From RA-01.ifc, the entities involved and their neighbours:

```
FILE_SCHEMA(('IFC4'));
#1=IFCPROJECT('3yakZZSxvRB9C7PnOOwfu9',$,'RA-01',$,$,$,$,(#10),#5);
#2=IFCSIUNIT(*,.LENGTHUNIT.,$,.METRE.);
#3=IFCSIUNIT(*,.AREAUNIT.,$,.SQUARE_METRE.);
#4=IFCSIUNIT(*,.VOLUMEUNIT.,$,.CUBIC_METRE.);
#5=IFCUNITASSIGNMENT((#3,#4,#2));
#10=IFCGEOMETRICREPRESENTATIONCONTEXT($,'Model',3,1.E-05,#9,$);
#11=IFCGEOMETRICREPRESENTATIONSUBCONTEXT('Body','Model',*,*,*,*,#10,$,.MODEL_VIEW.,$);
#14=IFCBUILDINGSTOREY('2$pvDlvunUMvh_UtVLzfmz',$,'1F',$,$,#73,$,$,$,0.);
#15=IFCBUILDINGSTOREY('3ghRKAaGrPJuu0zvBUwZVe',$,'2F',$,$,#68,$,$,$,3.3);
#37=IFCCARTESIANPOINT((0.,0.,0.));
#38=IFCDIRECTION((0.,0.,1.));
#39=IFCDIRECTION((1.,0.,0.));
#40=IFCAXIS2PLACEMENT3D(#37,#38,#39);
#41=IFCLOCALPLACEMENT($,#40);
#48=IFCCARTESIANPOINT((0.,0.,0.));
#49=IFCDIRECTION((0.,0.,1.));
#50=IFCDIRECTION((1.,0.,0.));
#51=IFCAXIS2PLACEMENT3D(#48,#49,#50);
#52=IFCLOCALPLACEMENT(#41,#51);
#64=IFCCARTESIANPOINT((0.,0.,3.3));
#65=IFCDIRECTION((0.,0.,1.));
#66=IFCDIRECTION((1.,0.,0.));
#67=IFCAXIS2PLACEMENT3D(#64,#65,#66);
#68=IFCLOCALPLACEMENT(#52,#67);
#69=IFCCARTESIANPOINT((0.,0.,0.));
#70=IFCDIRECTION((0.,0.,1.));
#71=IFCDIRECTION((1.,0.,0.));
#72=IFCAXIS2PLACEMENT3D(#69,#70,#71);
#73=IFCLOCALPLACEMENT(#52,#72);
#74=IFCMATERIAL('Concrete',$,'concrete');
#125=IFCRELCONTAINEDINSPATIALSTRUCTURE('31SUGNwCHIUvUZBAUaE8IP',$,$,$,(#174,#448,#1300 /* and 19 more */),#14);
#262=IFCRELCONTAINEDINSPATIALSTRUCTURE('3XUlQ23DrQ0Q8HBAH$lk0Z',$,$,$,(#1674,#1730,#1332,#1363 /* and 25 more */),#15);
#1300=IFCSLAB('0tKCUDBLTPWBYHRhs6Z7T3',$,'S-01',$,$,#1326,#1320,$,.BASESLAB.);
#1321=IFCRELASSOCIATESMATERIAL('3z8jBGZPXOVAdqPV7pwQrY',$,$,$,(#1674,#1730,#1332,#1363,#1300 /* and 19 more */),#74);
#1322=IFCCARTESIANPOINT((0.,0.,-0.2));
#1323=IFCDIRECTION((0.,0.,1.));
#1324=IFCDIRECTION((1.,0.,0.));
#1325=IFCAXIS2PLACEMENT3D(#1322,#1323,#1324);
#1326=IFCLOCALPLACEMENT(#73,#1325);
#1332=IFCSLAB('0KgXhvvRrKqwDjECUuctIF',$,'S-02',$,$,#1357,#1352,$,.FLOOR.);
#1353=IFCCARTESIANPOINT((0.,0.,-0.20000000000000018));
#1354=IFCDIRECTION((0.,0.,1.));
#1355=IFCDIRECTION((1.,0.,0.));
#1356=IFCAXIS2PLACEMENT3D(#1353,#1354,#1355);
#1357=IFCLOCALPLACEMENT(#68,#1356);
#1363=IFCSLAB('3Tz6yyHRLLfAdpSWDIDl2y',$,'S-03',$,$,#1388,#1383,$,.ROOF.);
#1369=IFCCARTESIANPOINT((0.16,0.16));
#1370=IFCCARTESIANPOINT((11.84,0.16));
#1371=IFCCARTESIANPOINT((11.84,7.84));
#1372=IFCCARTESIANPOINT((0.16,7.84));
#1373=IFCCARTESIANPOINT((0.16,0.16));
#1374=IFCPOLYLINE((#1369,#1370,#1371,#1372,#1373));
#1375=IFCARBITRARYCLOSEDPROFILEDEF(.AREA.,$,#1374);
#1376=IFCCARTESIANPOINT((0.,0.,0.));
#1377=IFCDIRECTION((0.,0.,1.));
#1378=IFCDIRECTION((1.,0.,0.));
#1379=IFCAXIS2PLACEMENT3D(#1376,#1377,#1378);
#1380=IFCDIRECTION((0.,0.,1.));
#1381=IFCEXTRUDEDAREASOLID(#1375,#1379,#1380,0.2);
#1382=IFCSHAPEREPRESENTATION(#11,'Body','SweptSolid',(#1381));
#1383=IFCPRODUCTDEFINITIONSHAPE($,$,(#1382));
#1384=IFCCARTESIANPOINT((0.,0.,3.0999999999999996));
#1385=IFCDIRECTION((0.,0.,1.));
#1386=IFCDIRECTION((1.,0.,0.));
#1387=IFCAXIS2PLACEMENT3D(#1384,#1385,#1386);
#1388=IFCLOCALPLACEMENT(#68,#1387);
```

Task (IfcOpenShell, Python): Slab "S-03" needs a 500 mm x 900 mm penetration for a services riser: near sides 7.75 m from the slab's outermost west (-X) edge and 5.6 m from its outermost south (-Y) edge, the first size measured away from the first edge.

```python
import numpy as np
import ifcopenshell
import ifcopenshell.api.feature
import ifcopenshell.api.geometry
import ifcopenshell.api.root
import ifcopenshell.geom
import ifcopenshell.util.placement
import ifcopenshell.util.representation
import ifcopenshell.util.shape
import ifcopenshell.util.unit

model = ifcopenshell.open("RA-01.ifc")
unit_scale = ifcopenshell.util.unit.calculate_unit_scale(model)
settings = ifcopenshell.geom.settings()


def volume(element):
    """Net volume in cubic metres, openings subtracted."""
    shape = ifcopenshell.geom.create_shape(settings, element)
    return ifcopenshell.util.shape.get_volume(shape.geometry)


slab = model.by_id(1363)
before = volume(slab)

# Extent in the slab's own axes, in metres. The edges named are its -X and -Y sides.
slab_shape = ifcopenshell.geom.create_shape(settings, slab)
vertices = ifcopenshell.util.shape.get_vertices(slab_shape.geometry)
x_min, y_min, bottom = vertices.min(axis=0)
top = vertices[:, 2].max()

opening = ifcopenshell.api.root.create_entity(model, ifc_class="IfcOpeningElement", name="Services riser opening", predefined_type="OPENING")
context = ifcopenshell.util.representation.get_context(model, "Model", "Body", "MODEL_VIEW")
width, depth = 0.5, 0.9
outline = [(0.0, 0.0), (width, 0.0), (width, depth), (0.0, depth), (0.0, 0.0)]
# Overshoot both faces by 50 mm so the cut is clean.
shape = ifcopenshell.api.geometry.add_slab_representation(
    model, context=context, depth=top - bottom + 0.1, polyline=outline
)
ifcopenshell.api.geometry.assign_representation(model, product=opening, representation=shape)

matrix = ifcopenshell.util.placement.get_local_placement(slab.ObjectPlacement)
matrix[:, 3] = matrix @ np.append(np.array([x_min + 7.75, y_min + 5.6, bottom - 0.05]) / unit_scale, 1.0)
ifcopenshell.api.geometry.edit_object_placement(model, product=opening, matrix=matrix, is_si=False)
ifcopenshell.api.feature.add_feature(model, feature=opening, element=slab)

after = volume(slab)

print(f"slab volume {before:.3f} -> {after:.3f} m3")

model.write("RA-01_updated.ifc")
```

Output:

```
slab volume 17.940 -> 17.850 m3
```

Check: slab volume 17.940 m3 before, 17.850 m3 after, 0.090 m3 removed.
